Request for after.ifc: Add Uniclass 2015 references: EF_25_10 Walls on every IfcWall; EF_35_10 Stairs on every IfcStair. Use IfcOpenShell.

First a look at what the model holds.

```python
import ifcopenshell

model = ifcopenshell.open("after.ifc")
print(model.schema)
print("classifications:", [c.Name for c in model.by_type("IfcClassification")])
for ifc_class in ("IfcDoor", "IfcRoof", "IfcStair", "IfcWall", "IfcWindow"):
    print(ifc_class, len(model.by_type(ifc_class)))
```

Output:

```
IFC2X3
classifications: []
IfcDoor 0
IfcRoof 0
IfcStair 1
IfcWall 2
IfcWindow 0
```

```python
import ifcopenshell
import ifcopenshell.api.classification

model = ifcopenshell.open("after.ifc")

# IFC2X3 requires Source and Edition and has no link from the project to the system.
system = model.create_entity("IfcClassification", Source="NBS", Edition="2015", Name="Uniclass 2015")

codes = {
    "IfcWall": ("EF_25_10", "Walls"),
    "IfcStair": ("EF_35_10", "Stairs"),
}
for ifc_class, (code, name) in codes.items():
    products = model.by_type(ifc_class)
    ifcopenshell.api.classification.add_reference(
        model, products=products, classification=system, identification=code, name=name
    )
    print(code, len(products))

model.write("after_rev.ifc")
```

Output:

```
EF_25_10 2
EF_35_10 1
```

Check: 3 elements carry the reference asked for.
